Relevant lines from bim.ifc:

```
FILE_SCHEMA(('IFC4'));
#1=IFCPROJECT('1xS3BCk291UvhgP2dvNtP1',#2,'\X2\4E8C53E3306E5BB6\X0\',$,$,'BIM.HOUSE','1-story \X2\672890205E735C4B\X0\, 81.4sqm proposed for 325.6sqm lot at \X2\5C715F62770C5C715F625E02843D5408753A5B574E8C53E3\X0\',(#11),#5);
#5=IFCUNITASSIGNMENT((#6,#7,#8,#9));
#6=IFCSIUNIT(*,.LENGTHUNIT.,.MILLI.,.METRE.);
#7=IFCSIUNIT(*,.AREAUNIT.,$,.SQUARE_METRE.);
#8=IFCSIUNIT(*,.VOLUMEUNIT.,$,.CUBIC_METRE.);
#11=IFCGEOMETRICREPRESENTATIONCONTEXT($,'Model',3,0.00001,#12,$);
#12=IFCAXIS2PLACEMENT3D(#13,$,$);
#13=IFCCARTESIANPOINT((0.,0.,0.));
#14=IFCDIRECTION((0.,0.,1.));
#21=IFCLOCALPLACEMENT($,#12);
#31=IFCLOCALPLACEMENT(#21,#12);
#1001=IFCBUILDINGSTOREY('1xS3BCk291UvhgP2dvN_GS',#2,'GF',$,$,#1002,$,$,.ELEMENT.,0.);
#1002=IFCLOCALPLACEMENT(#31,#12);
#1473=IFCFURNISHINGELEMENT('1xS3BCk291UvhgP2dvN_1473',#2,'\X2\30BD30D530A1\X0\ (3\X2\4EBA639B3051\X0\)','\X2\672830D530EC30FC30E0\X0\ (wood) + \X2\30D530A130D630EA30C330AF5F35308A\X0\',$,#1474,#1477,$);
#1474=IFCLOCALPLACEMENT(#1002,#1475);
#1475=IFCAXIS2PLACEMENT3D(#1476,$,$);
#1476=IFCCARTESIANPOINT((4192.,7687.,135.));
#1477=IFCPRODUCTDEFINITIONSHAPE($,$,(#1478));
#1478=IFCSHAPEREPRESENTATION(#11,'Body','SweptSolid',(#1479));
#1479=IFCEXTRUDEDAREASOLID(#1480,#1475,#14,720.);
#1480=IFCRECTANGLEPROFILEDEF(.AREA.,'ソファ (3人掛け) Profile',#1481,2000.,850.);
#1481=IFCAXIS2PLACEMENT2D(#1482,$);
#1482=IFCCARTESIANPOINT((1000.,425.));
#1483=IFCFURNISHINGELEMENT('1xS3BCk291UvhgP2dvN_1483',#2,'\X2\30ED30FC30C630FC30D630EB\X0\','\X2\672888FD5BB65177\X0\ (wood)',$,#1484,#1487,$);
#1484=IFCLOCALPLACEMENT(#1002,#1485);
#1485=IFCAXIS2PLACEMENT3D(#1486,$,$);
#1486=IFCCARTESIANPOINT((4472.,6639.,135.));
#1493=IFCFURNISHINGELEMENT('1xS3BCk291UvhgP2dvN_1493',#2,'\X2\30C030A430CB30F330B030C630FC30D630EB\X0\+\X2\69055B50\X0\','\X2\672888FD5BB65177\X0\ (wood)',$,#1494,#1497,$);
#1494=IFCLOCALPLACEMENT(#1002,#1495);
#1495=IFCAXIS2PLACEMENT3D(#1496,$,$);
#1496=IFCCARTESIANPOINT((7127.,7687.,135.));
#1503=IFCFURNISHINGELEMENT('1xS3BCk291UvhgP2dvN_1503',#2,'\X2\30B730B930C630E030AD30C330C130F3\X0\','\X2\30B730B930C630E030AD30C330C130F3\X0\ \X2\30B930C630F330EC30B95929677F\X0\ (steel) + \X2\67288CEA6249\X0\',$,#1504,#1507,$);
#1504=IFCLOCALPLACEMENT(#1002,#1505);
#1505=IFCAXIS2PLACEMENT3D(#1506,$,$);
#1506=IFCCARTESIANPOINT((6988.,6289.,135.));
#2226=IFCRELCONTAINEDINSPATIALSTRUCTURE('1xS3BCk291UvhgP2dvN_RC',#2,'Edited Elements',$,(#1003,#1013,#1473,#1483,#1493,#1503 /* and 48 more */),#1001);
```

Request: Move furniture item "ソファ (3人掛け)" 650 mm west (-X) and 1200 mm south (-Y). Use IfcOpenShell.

```python
import ifcopenshell
import ifcopenshell.api.geometry
import ifcopenshell.util.placement

model = ifcopenshell.open("bim.ifc")

item = model.by_guid("1xS3BCk291UvhgP2dvN_1473")
matrix = ifcopenshell.util.placement.get_local_placement(item.ObjectPlacement)
matrix[0, 3] -= 650.0
matrix[1, 3] -= 1200.0
ifcopenshell.api.geometry.edit_object_placement(model, product=item, matrix=matrix, is_si=False)

print(ifcopenshell.util.placement.get_local_placement(item.ObjectPlacement).round(3) + 0.0)

model.write("bim_v2.ifc")
```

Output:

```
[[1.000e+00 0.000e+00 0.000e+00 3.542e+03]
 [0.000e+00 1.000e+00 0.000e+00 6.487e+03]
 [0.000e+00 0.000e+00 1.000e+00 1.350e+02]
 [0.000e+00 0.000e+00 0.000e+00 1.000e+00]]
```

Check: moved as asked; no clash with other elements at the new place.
